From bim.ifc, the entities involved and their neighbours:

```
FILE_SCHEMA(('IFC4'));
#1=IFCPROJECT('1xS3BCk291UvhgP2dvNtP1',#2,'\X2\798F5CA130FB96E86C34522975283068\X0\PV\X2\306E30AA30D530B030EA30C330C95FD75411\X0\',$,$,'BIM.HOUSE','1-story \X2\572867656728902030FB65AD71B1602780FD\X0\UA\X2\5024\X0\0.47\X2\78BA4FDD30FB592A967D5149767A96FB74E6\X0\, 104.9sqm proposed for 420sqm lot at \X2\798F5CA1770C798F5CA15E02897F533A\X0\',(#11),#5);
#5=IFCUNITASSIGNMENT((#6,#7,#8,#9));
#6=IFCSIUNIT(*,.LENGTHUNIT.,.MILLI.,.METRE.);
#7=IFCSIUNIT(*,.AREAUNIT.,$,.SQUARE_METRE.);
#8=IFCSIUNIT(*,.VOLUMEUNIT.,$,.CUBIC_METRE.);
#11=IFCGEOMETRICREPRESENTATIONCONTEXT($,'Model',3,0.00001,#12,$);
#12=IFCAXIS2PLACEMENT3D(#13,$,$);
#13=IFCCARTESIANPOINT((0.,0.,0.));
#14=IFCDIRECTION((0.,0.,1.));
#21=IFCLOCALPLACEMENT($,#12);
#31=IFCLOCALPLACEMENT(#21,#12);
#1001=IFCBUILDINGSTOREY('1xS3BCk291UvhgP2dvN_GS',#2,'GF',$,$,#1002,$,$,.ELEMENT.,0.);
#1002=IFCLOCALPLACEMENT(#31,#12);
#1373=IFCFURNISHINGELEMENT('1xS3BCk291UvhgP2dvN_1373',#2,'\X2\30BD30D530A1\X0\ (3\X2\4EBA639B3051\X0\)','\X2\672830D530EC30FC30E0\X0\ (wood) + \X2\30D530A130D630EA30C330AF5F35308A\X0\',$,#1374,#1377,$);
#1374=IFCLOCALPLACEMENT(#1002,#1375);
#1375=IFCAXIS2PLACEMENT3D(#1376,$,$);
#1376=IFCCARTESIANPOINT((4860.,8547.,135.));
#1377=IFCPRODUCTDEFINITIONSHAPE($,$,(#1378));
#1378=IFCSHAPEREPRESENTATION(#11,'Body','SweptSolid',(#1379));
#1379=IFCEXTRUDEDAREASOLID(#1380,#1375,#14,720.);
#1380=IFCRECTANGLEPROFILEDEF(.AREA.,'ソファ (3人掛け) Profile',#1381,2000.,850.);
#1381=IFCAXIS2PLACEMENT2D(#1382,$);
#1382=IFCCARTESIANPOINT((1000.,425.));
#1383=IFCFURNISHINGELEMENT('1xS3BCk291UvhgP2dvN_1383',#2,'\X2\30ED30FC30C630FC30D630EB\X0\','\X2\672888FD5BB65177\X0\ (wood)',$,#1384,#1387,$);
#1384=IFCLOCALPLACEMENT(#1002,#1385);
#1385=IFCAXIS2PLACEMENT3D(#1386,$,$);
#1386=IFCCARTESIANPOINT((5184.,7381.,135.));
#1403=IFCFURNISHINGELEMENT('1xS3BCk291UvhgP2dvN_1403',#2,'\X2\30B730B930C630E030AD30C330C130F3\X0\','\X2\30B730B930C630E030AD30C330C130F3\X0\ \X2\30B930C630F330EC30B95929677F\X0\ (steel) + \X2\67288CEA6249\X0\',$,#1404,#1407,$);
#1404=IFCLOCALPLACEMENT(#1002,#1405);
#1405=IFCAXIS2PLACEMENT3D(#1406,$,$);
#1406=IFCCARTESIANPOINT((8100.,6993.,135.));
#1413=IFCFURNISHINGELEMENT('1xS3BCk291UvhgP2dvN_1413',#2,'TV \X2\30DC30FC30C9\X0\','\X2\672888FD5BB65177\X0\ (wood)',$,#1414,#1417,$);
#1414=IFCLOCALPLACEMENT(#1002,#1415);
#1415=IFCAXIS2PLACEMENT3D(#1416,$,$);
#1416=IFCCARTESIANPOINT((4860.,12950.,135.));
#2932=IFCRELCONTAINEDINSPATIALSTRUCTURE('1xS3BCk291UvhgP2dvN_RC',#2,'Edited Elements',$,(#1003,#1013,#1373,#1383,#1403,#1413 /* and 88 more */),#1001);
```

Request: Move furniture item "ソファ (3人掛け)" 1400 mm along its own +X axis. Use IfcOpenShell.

```python
import ifcopenshell
import ifcopenshell.api.geometry
import ifcopenshell.util.placement
import ifcopenshell.util.unit

model = ifcopenshell.open("bim.ifc")
unit_scale = ifcopenshell.util.unit.calculate_unit_scale(model)

item = model.by_guid("1xS3BCk291UvhgP2dvN_1373")
matrix = ifcopenshell.util.placement.get_local_placement(item.ObjectPlacement)
matrix[:3, 3] += matrix[:3, 0] * 1.4 / unit_scale
ifcopenshell.api.geometry.edit_object_placement(model, product=item, matrix=matrix, is_si=False)

print(ifcopenshell.util.placement.get_local_placement(item.ObjectPlacement).round(3) + 0.0)

model.write("bim_v2.ifc")
```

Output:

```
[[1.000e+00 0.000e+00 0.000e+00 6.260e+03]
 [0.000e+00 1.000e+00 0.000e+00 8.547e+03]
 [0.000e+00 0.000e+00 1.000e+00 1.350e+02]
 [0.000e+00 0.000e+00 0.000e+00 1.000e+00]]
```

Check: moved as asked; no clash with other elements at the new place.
